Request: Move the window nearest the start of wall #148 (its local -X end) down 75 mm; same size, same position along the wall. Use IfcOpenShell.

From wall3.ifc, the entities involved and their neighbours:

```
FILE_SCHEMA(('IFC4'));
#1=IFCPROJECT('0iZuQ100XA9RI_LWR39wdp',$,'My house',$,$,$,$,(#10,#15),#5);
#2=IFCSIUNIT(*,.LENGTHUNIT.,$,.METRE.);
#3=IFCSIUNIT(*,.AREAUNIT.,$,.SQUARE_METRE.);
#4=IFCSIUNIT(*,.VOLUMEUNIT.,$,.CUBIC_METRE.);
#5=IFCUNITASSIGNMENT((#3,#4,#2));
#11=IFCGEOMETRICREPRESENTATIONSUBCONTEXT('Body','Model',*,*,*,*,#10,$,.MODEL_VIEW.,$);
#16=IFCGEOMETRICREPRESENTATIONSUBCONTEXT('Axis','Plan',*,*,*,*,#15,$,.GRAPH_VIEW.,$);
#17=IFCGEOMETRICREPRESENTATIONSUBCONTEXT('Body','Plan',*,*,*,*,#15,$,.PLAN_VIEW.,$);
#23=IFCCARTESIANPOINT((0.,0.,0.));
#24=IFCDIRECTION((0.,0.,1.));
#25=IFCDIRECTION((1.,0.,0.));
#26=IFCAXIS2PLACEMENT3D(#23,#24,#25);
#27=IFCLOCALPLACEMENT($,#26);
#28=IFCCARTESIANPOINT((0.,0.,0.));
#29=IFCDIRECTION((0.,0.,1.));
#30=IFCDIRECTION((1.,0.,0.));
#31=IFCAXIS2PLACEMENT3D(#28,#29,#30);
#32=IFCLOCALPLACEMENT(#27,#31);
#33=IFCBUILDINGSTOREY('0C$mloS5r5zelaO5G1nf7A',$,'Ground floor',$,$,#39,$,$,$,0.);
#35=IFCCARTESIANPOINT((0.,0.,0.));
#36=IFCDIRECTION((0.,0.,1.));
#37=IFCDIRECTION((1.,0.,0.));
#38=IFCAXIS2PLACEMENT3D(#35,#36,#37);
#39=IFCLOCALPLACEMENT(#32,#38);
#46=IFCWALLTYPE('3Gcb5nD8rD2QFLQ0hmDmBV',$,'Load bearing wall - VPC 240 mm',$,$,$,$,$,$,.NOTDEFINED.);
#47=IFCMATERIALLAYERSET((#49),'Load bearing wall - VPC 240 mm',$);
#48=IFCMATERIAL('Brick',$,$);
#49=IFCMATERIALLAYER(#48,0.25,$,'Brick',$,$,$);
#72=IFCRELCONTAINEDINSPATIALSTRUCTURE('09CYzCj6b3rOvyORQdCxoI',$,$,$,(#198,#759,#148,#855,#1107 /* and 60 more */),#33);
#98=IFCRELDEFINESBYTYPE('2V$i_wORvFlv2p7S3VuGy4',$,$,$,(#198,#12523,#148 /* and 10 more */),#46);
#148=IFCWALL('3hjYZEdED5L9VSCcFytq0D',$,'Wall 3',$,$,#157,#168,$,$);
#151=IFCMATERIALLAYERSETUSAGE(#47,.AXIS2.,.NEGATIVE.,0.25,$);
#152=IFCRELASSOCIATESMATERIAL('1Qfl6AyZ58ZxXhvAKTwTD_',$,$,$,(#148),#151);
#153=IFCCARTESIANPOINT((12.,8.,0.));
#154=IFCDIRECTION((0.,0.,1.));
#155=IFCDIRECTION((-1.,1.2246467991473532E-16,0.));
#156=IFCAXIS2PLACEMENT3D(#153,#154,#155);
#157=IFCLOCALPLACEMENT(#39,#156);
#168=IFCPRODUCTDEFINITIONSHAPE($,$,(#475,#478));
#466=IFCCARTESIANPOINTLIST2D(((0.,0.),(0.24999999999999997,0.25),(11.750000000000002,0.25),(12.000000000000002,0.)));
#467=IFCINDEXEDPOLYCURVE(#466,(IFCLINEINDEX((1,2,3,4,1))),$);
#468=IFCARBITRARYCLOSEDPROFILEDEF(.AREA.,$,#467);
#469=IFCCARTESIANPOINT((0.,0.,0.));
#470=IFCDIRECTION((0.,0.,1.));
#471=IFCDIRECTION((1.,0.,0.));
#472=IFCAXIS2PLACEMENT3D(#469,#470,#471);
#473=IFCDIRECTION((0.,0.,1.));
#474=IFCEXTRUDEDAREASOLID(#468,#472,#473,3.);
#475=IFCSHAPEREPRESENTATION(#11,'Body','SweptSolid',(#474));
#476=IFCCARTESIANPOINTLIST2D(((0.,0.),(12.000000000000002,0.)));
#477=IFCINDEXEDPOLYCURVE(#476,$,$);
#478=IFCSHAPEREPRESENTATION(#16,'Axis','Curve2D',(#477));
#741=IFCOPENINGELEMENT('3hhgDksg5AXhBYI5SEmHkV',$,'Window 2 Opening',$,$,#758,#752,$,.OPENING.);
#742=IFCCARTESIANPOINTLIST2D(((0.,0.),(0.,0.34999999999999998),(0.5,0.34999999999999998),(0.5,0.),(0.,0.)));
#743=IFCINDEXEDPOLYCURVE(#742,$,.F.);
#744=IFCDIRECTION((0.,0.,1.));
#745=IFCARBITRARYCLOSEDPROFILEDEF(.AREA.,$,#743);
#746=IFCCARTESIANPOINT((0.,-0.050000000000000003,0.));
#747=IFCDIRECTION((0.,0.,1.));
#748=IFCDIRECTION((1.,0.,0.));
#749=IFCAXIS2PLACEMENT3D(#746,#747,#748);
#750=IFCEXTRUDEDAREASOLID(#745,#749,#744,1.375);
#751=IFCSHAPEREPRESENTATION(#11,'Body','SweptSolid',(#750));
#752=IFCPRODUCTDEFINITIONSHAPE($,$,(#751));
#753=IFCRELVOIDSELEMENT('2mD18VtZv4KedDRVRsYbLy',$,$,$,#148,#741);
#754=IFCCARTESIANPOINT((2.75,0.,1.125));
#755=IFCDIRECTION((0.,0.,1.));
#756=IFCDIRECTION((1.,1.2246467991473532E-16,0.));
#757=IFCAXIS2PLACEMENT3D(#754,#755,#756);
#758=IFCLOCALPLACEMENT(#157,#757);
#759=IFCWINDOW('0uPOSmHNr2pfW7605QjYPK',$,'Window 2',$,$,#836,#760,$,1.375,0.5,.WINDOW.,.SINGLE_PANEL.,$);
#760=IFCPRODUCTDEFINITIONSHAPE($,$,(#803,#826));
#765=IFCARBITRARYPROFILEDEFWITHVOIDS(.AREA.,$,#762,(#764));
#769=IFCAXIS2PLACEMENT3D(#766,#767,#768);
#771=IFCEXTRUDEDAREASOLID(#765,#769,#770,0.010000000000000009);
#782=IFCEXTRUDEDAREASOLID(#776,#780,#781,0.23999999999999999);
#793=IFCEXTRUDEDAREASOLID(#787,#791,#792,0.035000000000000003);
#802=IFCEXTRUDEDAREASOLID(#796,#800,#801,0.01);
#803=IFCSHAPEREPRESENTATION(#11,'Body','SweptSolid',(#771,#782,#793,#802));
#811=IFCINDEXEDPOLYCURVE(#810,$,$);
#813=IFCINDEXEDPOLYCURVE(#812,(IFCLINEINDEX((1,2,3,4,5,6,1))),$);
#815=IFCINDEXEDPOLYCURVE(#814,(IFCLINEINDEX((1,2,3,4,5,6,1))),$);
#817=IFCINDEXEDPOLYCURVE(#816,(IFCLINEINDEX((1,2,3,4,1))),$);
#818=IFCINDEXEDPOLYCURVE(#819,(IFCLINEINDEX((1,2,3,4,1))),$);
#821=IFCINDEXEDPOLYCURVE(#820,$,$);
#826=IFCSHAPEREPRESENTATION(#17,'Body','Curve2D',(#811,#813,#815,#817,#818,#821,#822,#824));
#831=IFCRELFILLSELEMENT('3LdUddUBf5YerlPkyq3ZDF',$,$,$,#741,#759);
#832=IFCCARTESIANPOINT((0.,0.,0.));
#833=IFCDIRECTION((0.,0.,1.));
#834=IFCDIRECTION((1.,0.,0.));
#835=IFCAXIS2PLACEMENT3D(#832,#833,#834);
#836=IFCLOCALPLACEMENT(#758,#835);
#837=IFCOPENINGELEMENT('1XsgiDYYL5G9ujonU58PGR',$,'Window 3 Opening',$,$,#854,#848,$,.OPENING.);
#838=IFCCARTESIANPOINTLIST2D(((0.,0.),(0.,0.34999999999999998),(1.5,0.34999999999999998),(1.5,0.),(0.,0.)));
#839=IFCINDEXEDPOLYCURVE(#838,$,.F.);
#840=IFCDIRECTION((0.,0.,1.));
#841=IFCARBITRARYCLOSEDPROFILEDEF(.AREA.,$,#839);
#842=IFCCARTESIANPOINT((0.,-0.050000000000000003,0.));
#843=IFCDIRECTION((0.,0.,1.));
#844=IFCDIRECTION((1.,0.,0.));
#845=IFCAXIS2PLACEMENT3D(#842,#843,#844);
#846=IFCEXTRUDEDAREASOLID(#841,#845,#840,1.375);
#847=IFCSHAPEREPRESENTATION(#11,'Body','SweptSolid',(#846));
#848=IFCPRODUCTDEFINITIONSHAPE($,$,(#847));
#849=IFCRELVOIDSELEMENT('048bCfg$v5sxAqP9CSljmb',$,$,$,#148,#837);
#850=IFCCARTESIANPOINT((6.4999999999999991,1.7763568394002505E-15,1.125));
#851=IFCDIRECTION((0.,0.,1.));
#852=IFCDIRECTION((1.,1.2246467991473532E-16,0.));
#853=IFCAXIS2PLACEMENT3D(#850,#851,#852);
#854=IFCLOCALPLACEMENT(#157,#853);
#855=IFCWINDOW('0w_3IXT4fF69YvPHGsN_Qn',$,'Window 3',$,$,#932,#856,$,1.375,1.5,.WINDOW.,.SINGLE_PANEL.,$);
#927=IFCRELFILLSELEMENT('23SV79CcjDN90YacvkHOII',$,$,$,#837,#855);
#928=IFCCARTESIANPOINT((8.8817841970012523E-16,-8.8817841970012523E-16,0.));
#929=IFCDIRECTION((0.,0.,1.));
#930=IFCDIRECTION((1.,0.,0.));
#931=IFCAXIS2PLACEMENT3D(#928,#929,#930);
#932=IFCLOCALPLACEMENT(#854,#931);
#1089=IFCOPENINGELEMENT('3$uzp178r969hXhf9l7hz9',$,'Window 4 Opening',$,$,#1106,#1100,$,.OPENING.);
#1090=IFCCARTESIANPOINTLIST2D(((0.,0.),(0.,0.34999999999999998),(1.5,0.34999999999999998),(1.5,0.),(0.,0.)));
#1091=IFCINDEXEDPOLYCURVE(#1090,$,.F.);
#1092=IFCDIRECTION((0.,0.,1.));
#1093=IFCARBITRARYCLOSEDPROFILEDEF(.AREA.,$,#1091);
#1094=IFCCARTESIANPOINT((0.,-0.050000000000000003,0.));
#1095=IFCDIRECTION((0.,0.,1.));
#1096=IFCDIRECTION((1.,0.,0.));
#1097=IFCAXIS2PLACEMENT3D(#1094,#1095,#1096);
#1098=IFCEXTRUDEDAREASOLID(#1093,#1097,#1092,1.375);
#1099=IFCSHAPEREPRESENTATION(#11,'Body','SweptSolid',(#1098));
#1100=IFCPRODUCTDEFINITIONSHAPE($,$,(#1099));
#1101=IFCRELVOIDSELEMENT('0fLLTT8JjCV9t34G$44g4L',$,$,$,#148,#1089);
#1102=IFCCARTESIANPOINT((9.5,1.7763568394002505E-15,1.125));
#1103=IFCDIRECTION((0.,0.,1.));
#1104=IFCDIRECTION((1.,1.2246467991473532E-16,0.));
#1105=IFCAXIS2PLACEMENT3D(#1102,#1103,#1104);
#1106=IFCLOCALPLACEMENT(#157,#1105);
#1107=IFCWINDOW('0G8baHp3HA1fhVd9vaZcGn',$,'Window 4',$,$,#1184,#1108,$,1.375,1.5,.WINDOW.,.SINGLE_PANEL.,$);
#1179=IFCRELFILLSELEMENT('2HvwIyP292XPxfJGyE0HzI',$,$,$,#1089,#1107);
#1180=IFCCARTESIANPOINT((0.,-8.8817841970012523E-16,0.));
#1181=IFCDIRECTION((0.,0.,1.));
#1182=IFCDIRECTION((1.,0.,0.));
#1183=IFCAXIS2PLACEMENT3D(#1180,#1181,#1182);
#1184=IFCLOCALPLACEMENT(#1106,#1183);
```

```python
import numpy as np
import ifcopenshell
import ifcopenshell.api.geometry
import ifcopenshell.util.placement
import ifcopenshell.util.unit

model = ifcopenshell.open("wall3.ifc")
unit_scale = ifcopenshell.util.unit.calculate_unit_scale(model)

window = model.by_guid("0uPOSmHNr2pfW7605QjYPK")
opening = window.FillsVoids[0].RelatingOpeningElement
dz = -0.075

shift = np.array([0.0, 0.0, dz])
# The window is placed relative to its opening, so it follows when the opening moves.
matrix = ifcopenshell.util.placement.get_local_placement(opening.ObjectPlacement)
matrix[:3, 3] += shift
ifcopenshell.api.geometry.edit_object_placement(
    model, product=opening, matrix=matrix, is_si=False, should_transform_children=True
)

print(f"moved by {dz * unit_scale:+.3f} m")

model.write("wall3_rev.ifc")
```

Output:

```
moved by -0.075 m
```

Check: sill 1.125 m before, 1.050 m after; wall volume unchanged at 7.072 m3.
